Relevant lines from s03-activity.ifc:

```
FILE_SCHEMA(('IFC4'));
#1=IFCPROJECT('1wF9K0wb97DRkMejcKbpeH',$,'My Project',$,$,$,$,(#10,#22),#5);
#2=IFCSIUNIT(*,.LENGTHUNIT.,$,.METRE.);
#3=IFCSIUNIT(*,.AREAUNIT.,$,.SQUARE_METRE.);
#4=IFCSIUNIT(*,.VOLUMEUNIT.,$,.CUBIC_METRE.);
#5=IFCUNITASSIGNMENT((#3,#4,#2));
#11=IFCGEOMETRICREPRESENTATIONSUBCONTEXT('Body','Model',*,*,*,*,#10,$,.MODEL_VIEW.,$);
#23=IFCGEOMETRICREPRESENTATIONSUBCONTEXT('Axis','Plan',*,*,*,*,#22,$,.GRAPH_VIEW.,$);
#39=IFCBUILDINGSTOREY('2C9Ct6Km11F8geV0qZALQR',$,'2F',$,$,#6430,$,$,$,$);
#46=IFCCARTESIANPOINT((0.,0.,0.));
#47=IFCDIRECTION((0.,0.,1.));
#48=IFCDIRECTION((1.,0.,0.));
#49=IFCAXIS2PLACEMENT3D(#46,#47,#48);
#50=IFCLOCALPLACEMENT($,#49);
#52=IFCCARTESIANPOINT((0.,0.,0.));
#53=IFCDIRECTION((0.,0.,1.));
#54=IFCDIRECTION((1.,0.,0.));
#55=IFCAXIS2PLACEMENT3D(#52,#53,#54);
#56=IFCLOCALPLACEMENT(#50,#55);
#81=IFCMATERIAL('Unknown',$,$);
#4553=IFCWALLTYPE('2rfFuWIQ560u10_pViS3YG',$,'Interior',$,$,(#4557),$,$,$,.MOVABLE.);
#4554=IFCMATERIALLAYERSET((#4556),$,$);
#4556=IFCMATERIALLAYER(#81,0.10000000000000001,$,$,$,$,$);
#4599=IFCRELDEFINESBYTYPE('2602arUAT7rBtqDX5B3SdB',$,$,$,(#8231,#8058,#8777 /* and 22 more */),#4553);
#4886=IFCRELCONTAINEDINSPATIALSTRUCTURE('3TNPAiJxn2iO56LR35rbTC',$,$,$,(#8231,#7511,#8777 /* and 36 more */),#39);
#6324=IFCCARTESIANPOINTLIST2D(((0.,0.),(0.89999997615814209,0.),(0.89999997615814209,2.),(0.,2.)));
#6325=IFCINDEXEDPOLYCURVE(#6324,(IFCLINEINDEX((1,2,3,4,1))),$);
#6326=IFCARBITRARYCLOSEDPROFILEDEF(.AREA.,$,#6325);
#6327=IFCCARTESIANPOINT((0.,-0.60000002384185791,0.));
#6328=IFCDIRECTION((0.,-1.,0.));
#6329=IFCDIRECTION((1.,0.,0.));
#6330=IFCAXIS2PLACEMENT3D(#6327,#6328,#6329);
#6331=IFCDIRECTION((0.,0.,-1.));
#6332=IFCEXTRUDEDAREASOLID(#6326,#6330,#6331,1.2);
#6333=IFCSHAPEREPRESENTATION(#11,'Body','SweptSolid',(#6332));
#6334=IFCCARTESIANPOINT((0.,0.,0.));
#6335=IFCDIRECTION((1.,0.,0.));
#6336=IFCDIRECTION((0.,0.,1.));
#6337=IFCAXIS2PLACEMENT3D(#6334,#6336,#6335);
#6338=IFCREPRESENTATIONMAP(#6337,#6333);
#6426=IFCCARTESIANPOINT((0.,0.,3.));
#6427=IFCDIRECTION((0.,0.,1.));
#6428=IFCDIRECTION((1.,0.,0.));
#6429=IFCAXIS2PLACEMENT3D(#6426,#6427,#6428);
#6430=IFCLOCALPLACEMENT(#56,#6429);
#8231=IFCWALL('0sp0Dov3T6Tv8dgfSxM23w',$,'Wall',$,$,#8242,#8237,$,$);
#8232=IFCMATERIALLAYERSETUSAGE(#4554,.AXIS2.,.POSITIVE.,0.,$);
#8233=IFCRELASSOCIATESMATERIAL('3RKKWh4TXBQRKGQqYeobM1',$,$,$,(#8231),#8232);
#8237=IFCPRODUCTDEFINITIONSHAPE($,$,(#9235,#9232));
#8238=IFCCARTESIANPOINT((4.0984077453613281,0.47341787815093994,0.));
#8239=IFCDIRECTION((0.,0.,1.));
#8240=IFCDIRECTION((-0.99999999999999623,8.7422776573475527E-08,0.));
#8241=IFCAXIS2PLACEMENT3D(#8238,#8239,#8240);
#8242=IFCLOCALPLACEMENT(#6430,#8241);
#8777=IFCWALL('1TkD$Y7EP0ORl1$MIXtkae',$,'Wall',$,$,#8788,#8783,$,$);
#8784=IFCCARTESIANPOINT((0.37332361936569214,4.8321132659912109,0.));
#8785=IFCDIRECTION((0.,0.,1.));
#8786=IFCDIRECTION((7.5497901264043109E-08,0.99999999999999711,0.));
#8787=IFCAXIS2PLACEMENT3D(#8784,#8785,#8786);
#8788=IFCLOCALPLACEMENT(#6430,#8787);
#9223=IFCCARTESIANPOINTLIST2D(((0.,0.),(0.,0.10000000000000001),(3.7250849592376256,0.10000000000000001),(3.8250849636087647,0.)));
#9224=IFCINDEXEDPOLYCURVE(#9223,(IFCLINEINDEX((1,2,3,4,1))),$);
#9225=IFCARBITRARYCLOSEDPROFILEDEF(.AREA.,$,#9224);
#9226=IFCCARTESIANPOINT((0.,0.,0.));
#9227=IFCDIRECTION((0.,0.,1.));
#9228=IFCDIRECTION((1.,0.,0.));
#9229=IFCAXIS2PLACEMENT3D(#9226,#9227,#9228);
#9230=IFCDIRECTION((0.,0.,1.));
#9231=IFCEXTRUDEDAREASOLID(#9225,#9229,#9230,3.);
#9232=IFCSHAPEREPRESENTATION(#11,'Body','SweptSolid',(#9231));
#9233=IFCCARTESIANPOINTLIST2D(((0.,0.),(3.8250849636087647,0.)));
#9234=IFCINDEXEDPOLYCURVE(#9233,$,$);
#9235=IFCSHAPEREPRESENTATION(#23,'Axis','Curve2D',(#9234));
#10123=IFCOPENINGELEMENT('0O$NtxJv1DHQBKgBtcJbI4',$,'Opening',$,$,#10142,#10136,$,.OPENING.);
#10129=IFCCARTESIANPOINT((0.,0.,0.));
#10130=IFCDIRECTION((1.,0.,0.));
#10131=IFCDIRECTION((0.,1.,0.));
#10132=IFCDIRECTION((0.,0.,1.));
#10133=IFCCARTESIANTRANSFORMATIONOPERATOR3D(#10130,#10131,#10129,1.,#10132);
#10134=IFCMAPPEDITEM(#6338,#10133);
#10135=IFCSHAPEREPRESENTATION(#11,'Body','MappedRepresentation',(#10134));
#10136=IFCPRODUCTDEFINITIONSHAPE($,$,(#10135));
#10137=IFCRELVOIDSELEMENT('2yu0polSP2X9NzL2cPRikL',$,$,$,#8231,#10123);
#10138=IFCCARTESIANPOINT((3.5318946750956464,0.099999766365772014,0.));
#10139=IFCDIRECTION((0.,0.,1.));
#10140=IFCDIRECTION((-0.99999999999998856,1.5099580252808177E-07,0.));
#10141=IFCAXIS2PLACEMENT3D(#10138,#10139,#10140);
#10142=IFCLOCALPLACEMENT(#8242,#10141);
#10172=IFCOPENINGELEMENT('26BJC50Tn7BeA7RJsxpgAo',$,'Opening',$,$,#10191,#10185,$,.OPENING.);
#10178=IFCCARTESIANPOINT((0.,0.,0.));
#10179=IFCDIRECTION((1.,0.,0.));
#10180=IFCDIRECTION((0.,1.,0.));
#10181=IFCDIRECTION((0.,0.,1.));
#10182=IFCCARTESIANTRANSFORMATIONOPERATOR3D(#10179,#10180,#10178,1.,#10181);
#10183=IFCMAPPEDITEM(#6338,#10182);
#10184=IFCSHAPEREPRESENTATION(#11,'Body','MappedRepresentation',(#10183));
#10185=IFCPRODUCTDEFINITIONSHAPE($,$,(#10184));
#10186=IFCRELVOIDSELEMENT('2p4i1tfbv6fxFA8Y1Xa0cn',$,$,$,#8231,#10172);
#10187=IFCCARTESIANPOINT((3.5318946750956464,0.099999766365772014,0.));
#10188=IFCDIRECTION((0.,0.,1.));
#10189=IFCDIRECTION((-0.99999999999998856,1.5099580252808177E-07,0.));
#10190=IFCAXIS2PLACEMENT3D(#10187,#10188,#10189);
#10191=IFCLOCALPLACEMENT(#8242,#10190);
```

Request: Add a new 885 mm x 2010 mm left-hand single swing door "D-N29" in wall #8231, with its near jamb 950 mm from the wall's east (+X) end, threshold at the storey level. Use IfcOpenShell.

```python
import numpy as np
import ifcopenshell
import ifcopenshell.api.feature
import ifcopenshell.api.geometry
import ifcopenshell.api.root
import ifcopenshell.api.spatial
import ifcopenshell.geom
import ifcopenshell.util.element
import ifcopenshell.util.placement
import ifcopenshell.util.representation
import ifcopenshell.util.shape
import ifcopenshell.util.unit

model = ifcopenshell.open("s03-activity.ifc")
unit_scale = ifcopenshell.util.unit.calculate_unit_scale(model)
settings = ifcopenshell.geom.settings()


def volume(element):
    """Net volume in cubic metres, openings subtracted."""
    shape = ifcopenshell.geom.create_shape(settings, element)
    return ifcopenshell.util.shape.get_volume(shape.geometry)


wall = model.by_guid("0sp0Dov3T6Tv8dgfSxM23w")
storey = ifcopenshell.util.element.get_container(wall, ifc_class="IfcBuildingStorey")
context = ifcopenshell.util.representation.get_context(model, "Model", "Body", "MODEL_VIEW")
before = volume(wall)

width, height, from_end, sill = 0.885, 2.01, 0.95, 0.0  # metres

# The wall runs along its own X axis, and the end named is its -X end.
wall_shape = ifcopenshell.geom.create_shape(settings, wall)
x, y, z = ifcopenshell.util.shape.get_vertices(wall_shape.geometry).T
start = x.min() + from_end
face, thickness = float(y.min()), float(y.max() - y.min())
wall_matrix = ifcopenshell.util.placement.get_local_placement(wall.ObjectPlacement)
level = ifcopenshell.util.placement.get_local_placement(storey.ObjectPlacement)[2, 3]


def in_wall(x, y):
    """Placement at x, y metres in the wall's axes, at sill height."""
    matrix = wall_matrix.copy()
    matrix[:, 3] = wall_matrix @ np.array([x / unit_scale, y / unit_scale, 0.0, 1.0])
    matrix[2, 3] = level + sill / unit_scale
    return matrix


# Opening: a box that overshoots both wall faces by 50 mm.
opening = ifcopenshell.api.root.create_entity(model, ifc_class="IfcOpeningElement", predefined_type="OPENING")
box = ifcopenshell.api.geometry.add_wall_representation(
    model, context=context, length=width, height=height, thickness=thickness + 0.1
)
ifcopenshell.api.geometry.assign_representation(model, product=opening, representation=box)
ifcopenshell.api.geometry.edit_object_placement(model, product=opening, matrix=in_wall(start, face - 0.05), is_si=False)
ifcopenshell.api.feature.add_feature(model, feature=opening, element=wall)

door = ifcopenshell.api.root.create_entity(model, ifc_class="IfcDoor", name="D-N29", predefined_type="DOOR")
door.OverallWidth, door.OverallHeight = width / unit_scale, height / unit_scale
door.OperationType = "SINGLE_SWING_LEFT"
body = ifcopenshell.api.geometry.add_door_representation(
    model,
    context=context,
    overall_width=door.OverallWidth,
    overall_height=door.OverallHeight,
    operation_type="SINGLE_SWING_LEFT",
    lining_properties={"LiningDepth": thickness / unit_scale, "ThresholdDepth": thickness / unit_scale},
)
ifcopenshell.api.geometry.assign_representation(model, product=door, representation=body)
ifcopenshell.api.spatial.assign_container(model, products=[door], relating_structure=storey)
ifcopenshell.api.feature.add_filling(model, opening=opening, element=door)

# The lining spans the wall, so the door starts at the wall face.
ifcopenshell.api.geometry.edit_object_placement(model, product=door, matrix=in_wall(start, face), is_si=False)

after = volume(wall)

print(f"wall volume {before:.3f} -> {after:.3f} m3")

model.write("s03-activity_updated.ifc")
```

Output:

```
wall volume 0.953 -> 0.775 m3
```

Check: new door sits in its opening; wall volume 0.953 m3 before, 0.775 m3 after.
